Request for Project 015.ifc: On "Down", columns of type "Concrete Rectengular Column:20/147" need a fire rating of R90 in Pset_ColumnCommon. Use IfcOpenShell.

First a look at what the model holds.

```python
import ifcopenshell
import ifcopenshell.util.element

model = ifcopenshell.open("Project 015.ifc")
print(model.schema)
storey = next(s for s in model.by_type("IfcBuildingStorey") if s.Name == "Down")
columns = [e for e in ifcopenshell.util.element.get_decomposition(storey) if e.is_a("IfcColumn")]
seen = {}
for e in columns:
    element_type = ifcopenshell.util.element.get_type(e)
    key = (element_type.Name if element_type != e and element_type else None, ifcopenshell.util.element.get_pset(e, "Pset_ColumnCommon", "FireRating"))
    seen[key] = seen.get(key, 0) + 1
for (name, value), count in sorted(seen.items(), key=str):
    print(count, "x", name, "|", value)
```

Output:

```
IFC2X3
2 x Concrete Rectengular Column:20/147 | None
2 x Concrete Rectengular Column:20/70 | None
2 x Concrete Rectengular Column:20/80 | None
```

```python
import ifcopenshell
import ifcopenshell.api.pset
import ifcopenshell.util.element

model = ifcopenshell.open("Project 015.ifc")

storey = next(s for s in model.by_type("IfcBuildingStorey") if s.Name == "Down")
columns = [e for e in ifcopenshell.util.element.get_decomposition(storey) if e.is_a("IfcColumn")]

count = 0
for e in columns:
    element_type = ifcopenshell.util.element.get_type(e)
    if element_type in (None, e) or element_type.Name != "Concrete Rectengular Column:20/147":
        continue
    # add_pset returns the element's existing set when there is one.
    pset = ifcopenshell.api.pset.add_pset(model, product=e, name="Pset_ColumnCommon")
    ifcopenshell.api.pset.edit_pset(model, pset=pset, properties={"FireRating": "R90"})
    count += 1

print(count, "columns updated")

model.write("Project 015-out.ifc")
```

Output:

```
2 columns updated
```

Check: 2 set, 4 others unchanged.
